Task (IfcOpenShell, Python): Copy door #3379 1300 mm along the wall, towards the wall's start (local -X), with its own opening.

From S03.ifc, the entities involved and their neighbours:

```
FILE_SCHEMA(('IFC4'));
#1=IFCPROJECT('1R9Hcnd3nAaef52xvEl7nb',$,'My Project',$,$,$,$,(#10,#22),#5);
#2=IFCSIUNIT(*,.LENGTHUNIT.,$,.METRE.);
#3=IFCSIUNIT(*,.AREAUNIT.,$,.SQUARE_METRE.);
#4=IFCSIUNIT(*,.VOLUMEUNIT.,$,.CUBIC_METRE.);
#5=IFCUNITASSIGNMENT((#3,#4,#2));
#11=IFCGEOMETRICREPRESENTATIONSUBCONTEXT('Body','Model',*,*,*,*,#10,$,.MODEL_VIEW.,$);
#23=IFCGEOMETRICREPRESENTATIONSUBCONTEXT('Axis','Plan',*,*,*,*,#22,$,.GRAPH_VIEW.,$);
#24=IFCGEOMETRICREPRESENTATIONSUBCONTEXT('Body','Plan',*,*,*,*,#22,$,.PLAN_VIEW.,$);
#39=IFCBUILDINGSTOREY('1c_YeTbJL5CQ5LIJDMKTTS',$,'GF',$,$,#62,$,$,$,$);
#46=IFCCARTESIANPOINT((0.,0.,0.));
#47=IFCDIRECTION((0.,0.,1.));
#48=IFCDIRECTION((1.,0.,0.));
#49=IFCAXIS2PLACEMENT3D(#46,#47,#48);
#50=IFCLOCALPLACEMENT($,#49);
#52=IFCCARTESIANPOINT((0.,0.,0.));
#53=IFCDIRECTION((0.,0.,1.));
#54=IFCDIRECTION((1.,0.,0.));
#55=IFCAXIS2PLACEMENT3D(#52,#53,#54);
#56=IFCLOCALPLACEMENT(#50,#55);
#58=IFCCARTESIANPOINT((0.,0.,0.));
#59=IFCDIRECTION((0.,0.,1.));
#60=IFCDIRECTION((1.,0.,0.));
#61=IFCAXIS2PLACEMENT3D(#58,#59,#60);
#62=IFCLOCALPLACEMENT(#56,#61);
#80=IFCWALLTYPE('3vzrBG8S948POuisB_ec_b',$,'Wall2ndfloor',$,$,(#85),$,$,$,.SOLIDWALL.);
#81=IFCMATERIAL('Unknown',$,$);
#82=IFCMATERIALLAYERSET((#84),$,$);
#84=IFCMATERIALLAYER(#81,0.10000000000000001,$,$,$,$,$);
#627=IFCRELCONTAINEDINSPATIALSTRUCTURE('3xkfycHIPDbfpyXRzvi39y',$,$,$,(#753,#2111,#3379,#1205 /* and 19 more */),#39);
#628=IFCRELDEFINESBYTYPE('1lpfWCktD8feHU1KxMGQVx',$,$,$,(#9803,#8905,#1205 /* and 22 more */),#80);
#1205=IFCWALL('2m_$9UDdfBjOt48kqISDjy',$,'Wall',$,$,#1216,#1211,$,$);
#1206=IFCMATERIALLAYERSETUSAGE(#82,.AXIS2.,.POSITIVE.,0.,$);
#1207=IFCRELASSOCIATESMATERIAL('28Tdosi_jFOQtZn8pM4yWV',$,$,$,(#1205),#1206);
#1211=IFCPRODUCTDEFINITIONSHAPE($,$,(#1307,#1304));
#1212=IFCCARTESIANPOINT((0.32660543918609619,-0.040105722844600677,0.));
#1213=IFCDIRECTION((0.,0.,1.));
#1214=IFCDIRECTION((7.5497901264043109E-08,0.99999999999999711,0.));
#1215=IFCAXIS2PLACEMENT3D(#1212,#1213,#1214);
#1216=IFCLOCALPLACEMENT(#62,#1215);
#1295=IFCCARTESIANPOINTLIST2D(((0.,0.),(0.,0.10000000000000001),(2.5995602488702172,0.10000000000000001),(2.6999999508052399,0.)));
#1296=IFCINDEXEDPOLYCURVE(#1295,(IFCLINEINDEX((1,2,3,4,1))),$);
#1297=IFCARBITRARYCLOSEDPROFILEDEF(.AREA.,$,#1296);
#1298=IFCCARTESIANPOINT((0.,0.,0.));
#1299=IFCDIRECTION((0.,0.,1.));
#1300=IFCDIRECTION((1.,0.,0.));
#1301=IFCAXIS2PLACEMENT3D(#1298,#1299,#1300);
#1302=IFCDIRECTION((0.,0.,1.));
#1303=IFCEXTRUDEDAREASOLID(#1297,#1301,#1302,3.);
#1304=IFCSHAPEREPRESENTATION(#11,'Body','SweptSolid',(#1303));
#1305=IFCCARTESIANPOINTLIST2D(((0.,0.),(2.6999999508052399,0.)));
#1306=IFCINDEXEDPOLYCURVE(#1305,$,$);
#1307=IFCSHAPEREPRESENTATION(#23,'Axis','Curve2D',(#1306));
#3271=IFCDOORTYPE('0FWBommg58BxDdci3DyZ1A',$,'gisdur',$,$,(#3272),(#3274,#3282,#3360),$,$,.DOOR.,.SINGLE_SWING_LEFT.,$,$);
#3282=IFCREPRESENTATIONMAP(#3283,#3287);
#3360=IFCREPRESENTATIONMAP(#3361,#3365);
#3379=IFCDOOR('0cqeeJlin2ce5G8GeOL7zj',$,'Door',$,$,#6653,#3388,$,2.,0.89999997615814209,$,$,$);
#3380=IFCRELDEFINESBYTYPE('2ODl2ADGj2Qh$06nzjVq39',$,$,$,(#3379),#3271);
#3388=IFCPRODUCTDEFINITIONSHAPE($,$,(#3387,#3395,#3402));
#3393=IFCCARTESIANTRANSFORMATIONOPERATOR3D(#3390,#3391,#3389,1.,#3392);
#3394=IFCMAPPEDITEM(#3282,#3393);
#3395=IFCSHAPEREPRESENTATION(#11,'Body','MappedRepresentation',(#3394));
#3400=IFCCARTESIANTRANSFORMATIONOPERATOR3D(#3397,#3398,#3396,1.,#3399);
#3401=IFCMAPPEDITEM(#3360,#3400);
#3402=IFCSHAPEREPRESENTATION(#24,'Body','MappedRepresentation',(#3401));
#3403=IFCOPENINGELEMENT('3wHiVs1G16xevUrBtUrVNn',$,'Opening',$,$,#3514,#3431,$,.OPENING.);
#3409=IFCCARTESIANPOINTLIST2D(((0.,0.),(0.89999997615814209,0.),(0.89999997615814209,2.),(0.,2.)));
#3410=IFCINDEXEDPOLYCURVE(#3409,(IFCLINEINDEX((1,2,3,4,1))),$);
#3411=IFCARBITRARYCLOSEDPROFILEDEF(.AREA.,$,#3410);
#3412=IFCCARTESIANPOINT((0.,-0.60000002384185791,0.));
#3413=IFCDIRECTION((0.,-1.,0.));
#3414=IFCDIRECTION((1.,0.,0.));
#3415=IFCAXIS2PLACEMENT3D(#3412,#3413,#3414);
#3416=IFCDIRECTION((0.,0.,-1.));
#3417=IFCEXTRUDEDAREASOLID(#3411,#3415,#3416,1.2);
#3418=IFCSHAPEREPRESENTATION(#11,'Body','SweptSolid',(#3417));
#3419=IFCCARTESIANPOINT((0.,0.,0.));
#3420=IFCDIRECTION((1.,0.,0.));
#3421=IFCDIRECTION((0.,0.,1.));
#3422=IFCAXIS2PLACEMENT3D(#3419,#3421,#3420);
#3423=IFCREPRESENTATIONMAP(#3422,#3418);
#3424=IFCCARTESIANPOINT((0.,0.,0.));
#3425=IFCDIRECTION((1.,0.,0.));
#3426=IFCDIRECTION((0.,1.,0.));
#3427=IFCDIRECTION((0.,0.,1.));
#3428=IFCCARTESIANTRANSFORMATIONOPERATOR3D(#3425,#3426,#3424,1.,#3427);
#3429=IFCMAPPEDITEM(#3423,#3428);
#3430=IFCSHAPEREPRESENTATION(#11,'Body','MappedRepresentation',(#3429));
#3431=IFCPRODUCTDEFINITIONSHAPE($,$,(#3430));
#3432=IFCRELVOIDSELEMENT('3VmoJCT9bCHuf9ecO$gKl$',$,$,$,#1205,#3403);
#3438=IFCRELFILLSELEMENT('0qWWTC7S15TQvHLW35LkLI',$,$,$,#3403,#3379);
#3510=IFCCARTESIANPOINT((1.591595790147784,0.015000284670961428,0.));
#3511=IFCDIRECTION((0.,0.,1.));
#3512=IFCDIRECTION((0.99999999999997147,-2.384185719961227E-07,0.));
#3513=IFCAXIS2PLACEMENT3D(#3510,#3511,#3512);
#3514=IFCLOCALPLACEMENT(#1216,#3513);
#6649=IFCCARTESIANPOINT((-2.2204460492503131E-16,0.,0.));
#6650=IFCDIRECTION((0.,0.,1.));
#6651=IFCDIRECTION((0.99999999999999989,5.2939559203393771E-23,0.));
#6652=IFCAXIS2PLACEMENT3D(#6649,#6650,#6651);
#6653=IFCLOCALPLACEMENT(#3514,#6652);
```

```python
import ifcopenshell
import ifcopenshell.api.feature
import ifcopenshell.api.geometry
import ifcopenshell.api.root
import ifcopenshell.geom
import ifcopenshell.util.element
import ifcopenshell.util.placement
import ifcopenshell.util.shape
import ifcopenshell.util.unit

model = ifcopenshell.open("S03.ifc")
unit_scale = ifcopenshell.util.unit.calculate_unit_scale(model)
settings = ifcopenshell.geom.settings()


def volume(element):
    """Net volume in cubic metres, openings subtracted."""
    shape = ifcopenshell.geom.create_shape(settings, element)
    return ifcopenshell.util.shape.get_volume(shape.geometry)


door = model.by_id(3379)
opening = door.FillsVoids[0].RelatingOpeningElement
wall = opening.VoidsElements[0].RelatingBuildingElement
before = volume(wall)
shift = ifcopenshell.util.placement.get_local_placement(wall.ObjectPlacement)[:3, 0] * -1.3 / unit_scale

# copy_class copies the void relationship, type, container and properties, but no geometry.
new_opening = ifcopenshell.api.root.copy_class(model, product=opening)
new_opening.Representation = ifcopenshell.util.element.copy_deep(
    model, opening.Representation, exclude=["IfcGeometricRepresentationContext", "IfcRepresentationMap"]
)
new_door = ifcopenshell.api.root.copy_class(model, product=door)
new_door.Representation = ifcopenshell.util.element.copy_deep(
    model, door.Representation, exclude=["IfcGeometricRepresentationContext", "IfcRepresentationMap"]
)
ifcopenshell.api.feature.add_filling(model, opening=new_opening, element=new_door)

for old, new in ((opening, new_opening), (door, new_door)):
    matrix = ifcopenshell.util.placement.get_local_placement(old.ObjectPlacement)
    matrix[:3, 3] += shift
    ifcopenshell.api.geometry.edit_object_placement(model, product=new, matrix=matrix, is_si=False)

after = volume(wall)

print(f"wall volume {before:.3f} -> {after:.3f} m3")

model.write("S03-out.ifc")
```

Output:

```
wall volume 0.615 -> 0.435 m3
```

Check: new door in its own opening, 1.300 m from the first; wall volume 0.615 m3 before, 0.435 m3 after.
